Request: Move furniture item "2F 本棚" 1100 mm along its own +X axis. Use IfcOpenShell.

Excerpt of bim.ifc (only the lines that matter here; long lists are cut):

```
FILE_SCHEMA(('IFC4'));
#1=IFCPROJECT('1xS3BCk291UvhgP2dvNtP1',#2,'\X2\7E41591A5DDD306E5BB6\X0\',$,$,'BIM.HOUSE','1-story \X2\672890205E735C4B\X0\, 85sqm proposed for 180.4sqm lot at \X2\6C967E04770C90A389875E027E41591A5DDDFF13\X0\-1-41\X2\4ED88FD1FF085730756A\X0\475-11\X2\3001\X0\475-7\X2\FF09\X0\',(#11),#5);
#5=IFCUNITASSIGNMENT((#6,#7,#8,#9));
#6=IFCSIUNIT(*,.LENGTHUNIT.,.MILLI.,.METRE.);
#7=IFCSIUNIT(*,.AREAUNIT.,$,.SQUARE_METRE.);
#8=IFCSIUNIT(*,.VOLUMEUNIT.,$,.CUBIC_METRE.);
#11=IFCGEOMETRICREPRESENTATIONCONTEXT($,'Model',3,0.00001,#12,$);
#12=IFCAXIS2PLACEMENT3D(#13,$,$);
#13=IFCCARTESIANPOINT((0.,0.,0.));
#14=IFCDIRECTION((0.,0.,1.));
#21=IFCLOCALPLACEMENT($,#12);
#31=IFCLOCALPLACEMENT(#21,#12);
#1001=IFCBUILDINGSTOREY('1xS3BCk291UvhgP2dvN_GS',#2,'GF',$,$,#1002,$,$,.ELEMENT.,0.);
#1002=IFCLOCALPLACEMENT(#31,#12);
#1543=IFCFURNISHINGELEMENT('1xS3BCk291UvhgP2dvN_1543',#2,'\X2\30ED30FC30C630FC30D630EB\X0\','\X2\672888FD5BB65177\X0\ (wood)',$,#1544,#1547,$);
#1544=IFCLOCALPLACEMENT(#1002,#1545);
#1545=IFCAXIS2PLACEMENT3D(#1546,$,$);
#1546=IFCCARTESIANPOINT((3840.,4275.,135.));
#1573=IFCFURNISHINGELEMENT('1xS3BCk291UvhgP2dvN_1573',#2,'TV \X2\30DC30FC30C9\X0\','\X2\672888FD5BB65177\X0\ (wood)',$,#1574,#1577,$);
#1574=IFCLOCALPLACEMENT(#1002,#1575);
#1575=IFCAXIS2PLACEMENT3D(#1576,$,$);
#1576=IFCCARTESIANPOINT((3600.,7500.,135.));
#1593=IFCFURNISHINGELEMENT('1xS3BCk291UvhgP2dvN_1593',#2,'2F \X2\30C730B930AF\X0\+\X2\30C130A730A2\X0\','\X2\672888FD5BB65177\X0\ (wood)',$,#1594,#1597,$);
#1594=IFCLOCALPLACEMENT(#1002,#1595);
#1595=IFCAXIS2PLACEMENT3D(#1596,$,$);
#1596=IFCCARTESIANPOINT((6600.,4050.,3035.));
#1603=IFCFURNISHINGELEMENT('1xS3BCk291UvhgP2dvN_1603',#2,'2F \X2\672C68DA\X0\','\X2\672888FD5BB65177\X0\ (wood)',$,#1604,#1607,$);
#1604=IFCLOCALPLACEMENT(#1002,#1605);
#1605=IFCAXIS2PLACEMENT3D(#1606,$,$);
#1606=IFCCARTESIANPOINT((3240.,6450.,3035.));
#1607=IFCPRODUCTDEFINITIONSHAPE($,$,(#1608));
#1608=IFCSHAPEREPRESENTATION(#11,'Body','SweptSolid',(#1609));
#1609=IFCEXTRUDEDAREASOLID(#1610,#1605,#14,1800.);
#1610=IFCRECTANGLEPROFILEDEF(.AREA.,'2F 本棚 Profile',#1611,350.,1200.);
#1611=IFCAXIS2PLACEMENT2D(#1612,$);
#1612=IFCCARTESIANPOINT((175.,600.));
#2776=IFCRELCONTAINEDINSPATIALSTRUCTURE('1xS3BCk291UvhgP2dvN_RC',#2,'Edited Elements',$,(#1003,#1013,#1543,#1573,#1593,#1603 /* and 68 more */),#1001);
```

```python
import ifcopenshell
import ifcopenshell.api.geometry
import ifcopenshell.util.placement

model = ifcopenshell.open("bim.ifc")

item = model.by_guid("1xS3BCk291UvhgP2dvN_1603")
matrix = ifcopenshell.util.placement.get_local_placement(item.ObjectPlacement)
matrix[:3, 3] += matrix[:3, 0] * 1100.0
ifcopenshell.api.geometry.edit_object_placement(model, product=item, matrix=matrix, is_si=False)

print(ifcopenshell.util.placement.get_local_placement(item.ObjectPlacement).round(3) + 0.0)

model.write("bim_updated.ifc")
```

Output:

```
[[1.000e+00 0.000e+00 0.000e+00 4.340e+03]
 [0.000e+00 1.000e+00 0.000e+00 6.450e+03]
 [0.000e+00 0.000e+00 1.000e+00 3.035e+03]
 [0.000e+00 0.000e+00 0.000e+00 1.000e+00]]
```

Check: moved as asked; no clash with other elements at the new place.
